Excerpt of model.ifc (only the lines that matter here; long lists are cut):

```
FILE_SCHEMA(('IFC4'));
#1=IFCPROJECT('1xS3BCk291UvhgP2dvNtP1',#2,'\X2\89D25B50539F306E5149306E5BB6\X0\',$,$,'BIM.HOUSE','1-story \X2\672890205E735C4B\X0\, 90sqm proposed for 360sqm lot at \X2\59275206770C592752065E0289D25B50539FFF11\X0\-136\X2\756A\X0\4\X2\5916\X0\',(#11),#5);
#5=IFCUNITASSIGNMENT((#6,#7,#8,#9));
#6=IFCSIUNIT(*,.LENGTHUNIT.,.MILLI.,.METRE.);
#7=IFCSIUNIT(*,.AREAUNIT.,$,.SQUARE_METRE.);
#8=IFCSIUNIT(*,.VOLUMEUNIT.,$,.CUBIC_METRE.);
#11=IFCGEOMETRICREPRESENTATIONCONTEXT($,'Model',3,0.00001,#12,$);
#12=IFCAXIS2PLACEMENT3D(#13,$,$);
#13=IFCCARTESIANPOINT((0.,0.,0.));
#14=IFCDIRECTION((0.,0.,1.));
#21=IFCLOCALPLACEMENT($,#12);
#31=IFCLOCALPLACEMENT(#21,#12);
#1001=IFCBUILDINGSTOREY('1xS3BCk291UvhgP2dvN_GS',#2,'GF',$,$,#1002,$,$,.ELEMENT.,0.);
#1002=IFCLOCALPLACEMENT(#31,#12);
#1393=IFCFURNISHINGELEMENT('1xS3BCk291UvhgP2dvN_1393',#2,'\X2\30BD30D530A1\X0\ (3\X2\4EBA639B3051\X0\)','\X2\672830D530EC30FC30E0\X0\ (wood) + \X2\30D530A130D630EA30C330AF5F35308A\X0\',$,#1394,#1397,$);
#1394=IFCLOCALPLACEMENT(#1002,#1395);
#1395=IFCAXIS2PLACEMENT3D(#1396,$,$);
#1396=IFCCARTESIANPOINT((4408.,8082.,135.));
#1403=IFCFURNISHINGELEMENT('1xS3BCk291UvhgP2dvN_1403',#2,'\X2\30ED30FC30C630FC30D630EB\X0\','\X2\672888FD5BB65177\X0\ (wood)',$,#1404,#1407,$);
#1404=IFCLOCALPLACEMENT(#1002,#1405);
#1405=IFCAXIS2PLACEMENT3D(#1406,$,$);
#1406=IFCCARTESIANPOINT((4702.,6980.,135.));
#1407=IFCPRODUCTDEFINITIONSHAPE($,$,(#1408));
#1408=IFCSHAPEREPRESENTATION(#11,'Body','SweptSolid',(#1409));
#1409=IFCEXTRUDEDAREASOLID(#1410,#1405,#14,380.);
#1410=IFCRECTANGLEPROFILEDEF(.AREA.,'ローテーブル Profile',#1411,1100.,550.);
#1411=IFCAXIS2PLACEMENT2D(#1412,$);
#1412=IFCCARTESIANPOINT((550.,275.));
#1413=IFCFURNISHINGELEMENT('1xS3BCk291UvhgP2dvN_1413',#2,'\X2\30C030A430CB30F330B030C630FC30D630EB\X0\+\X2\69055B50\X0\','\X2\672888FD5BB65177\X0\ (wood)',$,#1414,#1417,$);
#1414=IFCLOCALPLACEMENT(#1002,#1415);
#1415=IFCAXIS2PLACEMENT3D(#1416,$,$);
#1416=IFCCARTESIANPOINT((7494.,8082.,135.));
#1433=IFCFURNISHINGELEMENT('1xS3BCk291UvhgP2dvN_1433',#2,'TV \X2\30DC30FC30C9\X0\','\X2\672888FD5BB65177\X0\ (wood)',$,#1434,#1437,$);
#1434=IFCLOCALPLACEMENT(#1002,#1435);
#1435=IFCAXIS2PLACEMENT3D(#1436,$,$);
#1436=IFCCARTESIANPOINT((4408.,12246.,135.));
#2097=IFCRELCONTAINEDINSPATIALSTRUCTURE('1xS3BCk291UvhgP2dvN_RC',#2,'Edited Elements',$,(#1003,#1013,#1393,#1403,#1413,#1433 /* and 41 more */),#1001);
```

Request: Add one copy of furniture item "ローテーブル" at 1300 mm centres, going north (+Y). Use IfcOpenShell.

```python
import numpy as np
import ifcopenshell
import ifcopenshell.api.geometry
import ifcopenshell.api.root
import ifcopenshell.util.element
import ifcopenshell.util.placement

model = ifcopenshell.open("model.ifc")


def reuse_history(source, copy):
    """copy_class also copies each property set's owner history, people and application; keep the originals."""
    for rel in copy.IsDefinedBy:
        if rel.is_a("IfcRelDefinesByProperties") and (history := rel.RelatingPropertyDefinition.OwnerHistory):
            rel.RelatingPropertyDefinition.OwnerHistory = source.OwnerHistory
            ifcopenshell.util.element.remove_deep2(model, history)


source = model.by_guid("1xS3BCk291UvhgP2dvN_1403")
base = ifcopenshell.util.placement.get_local_placement(source.ObjectPlacement)
step = np.array([0.0, 1.0, 0.0]) * 1300.0

for i in range(1, 2):
    copy = ifcopenshell.api.root.copy_class(model, product=source)
    copy.Representation = ifcopenshell.util.element.copy_deep(
        model, source.Representation, exclude=["IfcGeometricRepresentationContext", "IfcRepresentationMap"]
    )
    reuse_history(source, copy)
    matrix = base.copy()
    matrix[:3, 3] += i * step
    print("added at", matrix[:3, 3].round(3) + 0.0)
    ifcopenshell.api.geometry.edit_object_placement(model, product=copy, matrix=matrix, is_si=False)

model.write("model_v2.ifc")
```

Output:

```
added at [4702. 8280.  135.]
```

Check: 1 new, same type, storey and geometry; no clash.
